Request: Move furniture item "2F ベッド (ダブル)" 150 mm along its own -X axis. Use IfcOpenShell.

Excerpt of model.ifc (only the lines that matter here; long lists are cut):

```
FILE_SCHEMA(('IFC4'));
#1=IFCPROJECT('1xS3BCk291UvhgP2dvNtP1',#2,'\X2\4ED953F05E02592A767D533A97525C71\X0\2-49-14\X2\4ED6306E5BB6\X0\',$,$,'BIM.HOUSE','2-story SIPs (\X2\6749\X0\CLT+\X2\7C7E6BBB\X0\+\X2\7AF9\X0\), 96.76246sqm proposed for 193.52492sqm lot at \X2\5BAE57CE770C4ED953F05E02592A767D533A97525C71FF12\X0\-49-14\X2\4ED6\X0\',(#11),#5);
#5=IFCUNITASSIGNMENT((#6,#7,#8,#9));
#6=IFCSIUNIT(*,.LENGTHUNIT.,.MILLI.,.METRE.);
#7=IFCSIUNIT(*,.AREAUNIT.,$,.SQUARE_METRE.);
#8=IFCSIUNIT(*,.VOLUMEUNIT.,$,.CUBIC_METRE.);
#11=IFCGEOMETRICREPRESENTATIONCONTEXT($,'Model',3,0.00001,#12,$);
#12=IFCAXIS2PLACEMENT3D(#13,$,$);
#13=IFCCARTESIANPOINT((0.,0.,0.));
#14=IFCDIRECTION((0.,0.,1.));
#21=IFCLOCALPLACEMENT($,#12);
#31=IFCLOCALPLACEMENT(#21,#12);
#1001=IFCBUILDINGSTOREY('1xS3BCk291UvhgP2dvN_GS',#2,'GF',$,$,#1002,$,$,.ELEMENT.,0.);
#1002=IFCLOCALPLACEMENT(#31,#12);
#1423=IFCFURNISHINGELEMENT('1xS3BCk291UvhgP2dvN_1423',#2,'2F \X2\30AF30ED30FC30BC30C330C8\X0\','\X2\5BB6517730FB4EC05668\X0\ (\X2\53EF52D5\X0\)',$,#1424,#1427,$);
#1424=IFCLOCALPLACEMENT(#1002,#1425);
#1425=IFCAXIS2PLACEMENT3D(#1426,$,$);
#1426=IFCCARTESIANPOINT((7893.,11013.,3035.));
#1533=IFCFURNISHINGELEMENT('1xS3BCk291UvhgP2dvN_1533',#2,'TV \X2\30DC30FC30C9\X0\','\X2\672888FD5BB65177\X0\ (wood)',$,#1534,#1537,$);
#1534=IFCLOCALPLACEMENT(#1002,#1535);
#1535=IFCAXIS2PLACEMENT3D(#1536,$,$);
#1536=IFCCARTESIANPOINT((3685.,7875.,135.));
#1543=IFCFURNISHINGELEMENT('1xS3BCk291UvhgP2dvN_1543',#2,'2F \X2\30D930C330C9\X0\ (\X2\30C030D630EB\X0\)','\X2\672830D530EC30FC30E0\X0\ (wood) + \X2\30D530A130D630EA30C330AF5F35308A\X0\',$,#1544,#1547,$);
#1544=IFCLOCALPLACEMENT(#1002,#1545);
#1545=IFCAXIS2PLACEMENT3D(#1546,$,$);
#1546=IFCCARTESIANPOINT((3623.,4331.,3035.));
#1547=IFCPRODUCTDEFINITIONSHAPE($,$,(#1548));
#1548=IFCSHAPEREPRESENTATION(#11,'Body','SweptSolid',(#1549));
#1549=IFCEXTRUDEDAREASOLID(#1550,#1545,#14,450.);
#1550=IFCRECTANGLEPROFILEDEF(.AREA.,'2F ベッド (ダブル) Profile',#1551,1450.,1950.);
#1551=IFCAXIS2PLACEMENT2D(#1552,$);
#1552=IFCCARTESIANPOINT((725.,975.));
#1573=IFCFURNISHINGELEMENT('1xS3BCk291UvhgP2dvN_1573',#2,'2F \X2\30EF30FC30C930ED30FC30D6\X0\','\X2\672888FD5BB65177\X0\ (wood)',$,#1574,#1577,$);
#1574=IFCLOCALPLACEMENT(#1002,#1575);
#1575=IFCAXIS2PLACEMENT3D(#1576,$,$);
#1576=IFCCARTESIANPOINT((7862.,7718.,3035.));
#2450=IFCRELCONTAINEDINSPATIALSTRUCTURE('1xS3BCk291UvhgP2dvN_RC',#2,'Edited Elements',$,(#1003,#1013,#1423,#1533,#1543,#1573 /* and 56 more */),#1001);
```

```python
import ifcopenshell
import ifcopenshell.api.geometry
import ifcopenshell.util.placement

model = ifcopenshell.open("model.ifc")

item = model.by_guid("1xS3BCk291UvhgP2dvN_1543")
matrix = ifcopenshell.util.placement.get_local_placement(item.ObjectPlacement)
matrix[:3, 3] -= matrix[:3, 0] * 150.0
ifcopenshell.api.geometry.edit_object_placement(model, product=item, matrix=matrix, is_si=False)

print(ifcopenshell.util.placement.get_local_placement(item.ObjectPlacement).round(3) + 0.0)

model.write("model_updated.ifc")
```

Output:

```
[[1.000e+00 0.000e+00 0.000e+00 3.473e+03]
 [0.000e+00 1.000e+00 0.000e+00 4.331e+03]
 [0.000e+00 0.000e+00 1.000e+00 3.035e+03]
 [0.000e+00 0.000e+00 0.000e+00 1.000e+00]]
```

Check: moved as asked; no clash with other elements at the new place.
